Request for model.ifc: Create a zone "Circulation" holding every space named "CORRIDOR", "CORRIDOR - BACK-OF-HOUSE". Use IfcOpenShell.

First a look at what the model holds.

```python
import ifcopenshell

model = ifcopenshell.open("model.ifc")
print(model.schema)
seen = {}
for space in model.by_type("IfcSpace"):
    seen[space.LongName] = seen.get(space.LongName, 0) + 1
for name, count in sorted(seen.items(), key=str):
    print(count, "x", name)
print("zones:", [z.Name for z in model.by_type("IfcZone")][:20])
```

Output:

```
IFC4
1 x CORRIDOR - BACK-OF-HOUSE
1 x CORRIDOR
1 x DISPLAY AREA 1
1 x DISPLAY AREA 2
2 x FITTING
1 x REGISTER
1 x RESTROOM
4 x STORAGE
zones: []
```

```python
import ifcopenshell
import ifcopenshell.api.group
import ifcopenshell.api.root

model = ifcopenshell.open("model.ifc")

names = {"CORRIDOR", "CORRIDOR - BACK-OF-HOUSE"}
spaces = [s for s in model.by_type("IfcSpace") if s.LongName in names]

zone = ifcopenshell.api.root.create_entity(model, ifc_class="IfcZone", name="Circulation")
ifcopenshell.api.group.assign_group(model, products=spaces, group=zone)
print(len(spaces), "spaces in", zone.Name)

model.write("model_v2.ifc")
```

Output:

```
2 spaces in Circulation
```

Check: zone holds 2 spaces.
